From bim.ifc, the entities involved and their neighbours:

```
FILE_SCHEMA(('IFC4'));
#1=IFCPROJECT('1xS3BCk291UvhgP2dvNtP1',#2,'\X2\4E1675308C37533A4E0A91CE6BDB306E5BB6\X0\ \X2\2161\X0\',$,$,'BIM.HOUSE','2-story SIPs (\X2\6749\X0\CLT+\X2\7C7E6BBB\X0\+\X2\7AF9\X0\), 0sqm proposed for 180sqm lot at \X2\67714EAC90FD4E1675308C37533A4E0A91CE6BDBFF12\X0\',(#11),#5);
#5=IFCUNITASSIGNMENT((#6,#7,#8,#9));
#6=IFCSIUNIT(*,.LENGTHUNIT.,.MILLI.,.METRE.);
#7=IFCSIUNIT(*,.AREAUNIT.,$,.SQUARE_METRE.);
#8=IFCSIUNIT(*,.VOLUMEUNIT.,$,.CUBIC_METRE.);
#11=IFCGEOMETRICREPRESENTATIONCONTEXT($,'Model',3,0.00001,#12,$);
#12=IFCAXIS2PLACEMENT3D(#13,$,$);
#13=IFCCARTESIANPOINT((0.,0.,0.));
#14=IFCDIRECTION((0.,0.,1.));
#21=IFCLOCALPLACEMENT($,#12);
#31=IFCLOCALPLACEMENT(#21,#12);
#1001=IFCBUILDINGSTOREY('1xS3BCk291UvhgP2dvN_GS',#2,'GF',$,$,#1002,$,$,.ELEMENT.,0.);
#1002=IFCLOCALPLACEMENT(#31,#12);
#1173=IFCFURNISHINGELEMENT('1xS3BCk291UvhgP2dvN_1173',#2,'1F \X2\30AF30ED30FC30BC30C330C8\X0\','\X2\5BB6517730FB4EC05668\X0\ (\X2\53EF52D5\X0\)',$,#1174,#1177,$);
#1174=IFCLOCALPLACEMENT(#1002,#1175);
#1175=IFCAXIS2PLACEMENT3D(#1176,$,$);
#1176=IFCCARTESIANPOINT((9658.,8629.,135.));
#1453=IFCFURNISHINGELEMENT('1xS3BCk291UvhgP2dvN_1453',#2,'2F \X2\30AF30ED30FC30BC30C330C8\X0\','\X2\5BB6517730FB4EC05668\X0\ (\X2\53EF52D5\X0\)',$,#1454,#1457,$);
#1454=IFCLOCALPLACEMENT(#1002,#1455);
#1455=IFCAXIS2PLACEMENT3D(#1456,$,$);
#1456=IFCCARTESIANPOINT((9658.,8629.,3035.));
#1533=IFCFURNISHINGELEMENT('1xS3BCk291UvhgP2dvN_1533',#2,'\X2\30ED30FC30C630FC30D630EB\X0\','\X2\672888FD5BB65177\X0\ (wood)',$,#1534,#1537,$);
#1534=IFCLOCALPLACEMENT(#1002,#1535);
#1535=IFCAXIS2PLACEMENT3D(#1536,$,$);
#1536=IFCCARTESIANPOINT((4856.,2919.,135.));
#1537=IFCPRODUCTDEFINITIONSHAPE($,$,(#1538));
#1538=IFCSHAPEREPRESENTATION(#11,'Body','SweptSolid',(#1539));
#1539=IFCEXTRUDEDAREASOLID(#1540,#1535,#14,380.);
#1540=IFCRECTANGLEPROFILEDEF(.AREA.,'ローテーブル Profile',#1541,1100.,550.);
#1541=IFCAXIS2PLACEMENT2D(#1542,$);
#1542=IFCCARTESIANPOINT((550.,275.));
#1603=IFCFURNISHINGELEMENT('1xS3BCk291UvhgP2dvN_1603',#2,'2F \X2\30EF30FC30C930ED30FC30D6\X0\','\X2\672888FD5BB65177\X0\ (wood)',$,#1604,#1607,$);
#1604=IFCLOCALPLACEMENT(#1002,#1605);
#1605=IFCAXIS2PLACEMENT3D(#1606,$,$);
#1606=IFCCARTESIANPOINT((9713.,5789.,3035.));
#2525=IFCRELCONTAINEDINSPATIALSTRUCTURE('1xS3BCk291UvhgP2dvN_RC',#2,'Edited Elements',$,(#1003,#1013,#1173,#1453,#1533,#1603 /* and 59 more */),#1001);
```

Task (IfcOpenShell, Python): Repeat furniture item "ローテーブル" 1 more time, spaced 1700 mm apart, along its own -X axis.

```python
import ifcopenshell
import ifcopenshell.api.geometry
import ifcopenshell.api.root
import ifcopenshell.util.element
import ifcopenshell.util.placement

model = ifcopenshell.open("bim.ifc")


def reuse_history(source, copy):
    """copy_class also copies each property set's owner history, people and application; keep the originals."""
    for rel in copy.IsDefinedBy:
        if rel.is_a("IfcRelDefinesByProperties") and (history := rel.RelatingPropertyDefinition.OwnerHistory):
            rel.RelatingPropertyDefinition.OwnerHistory = source.OwnerHistory
            ifcopenshell.util.element.remove_deep2(model, history)


source = model.by_guid("1xS3BCk291UvhgP2dvN_1533")
base = ifcopenshell.util.placement.get_local_placement(source.ObjectPlacement)
step = -base[:3, 0] * 1700.0

for i in range(1, 2):
    copy = ifcopenshell.api.root.copy_class(model, product=source)
    copy.Representation = ifcopenshell.util.element.copy_deep(
        model, source.Representation, exclude=["IfcGeometricRepresentationContext", "IfcRepresentationMap"]
    )
    reuse_history(source, copy)
    matrix = base.copy()
    matrix[:3, 3] += i * step
    print("added at", matrix[:3, 3].round(3) + 0.0)
    ifcopenshell.api.geometry.edit_object_placement(model, product=copy, matrix=matrix, is_si=False)

model.write("bim_edited.ifc")
```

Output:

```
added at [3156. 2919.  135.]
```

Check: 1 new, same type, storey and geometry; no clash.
